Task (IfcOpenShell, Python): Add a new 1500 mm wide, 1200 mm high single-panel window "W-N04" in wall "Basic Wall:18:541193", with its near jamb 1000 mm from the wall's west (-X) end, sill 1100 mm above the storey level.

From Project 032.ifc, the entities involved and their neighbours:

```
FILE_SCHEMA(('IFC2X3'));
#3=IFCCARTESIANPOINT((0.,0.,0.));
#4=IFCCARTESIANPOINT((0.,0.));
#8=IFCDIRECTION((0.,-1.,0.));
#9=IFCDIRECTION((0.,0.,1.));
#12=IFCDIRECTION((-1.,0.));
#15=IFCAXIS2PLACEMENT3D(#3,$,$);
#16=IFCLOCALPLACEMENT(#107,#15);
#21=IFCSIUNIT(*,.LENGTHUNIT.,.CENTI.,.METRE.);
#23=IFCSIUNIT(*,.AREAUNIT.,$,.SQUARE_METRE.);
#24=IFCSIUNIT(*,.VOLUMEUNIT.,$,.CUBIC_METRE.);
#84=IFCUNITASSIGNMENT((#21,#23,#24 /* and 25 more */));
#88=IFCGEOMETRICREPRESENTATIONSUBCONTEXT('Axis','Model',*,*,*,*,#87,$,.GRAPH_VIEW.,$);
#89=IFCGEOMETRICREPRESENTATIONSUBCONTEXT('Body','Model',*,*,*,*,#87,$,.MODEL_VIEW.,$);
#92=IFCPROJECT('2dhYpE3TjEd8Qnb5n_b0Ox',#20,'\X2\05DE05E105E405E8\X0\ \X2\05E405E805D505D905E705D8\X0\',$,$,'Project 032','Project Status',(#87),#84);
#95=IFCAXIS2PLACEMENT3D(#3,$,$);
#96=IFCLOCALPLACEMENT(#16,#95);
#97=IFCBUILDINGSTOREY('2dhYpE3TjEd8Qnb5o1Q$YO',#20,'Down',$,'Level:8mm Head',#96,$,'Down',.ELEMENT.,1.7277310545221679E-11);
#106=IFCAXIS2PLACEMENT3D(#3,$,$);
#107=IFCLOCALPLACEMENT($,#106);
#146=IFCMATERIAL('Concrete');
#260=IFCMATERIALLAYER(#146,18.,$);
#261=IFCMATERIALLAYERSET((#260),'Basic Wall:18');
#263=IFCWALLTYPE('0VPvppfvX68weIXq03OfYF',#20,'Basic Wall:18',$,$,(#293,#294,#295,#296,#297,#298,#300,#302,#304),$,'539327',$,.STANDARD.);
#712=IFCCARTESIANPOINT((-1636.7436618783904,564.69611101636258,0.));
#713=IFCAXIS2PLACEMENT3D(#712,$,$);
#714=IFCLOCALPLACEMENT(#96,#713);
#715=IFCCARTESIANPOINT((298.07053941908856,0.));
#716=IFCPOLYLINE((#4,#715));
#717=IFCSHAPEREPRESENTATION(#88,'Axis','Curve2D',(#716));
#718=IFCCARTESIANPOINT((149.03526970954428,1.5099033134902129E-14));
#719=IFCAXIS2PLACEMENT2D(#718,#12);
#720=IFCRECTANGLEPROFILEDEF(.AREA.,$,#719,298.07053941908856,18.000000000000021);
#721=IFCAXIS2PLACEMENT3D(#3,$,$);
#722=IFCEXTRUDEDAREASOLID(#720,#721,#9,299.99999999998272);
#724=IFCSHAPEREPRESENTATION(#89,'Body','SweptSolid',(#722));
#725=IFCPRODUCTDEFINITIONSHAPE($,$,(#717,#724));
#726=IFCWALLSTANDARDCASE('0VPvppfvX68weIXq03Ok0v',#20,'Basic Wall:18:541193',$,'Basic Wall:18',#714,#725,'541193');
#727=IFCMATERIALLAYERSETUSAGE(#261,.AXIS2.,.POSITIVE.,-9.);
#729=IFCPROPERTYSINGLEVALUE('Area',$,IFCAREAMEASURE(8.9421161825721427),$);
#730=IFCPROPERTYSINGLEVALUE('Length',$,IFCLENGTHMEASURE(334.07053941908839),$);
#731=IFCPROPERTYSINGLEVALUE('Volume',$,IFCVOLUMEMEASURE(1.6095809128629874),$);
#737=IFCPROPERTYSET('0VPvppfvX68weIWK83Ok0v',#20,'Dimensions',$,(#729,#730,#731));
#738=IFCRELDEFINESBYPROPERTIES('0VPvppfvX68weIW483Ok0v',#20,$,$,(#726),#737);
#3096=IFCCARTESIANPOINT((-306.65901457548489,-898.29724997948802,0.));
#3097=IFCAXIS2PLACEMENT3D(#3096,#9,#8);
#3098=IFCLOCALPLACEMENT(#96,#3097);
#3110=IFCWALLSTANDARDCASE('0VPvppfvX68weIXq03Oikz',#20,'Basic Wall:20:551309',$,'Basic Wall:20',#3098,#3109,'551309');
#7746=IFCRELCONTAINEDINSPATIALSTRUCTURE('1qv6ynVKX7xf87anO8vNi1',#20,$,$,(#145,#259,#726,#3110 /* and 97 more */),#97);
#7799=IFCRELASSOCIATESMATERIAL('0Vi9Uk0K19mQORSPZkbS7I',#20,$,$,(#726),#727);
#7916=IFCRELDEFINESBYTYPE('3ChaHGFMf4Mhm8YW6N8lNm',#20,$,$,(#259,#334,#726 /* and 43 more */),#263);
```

```python
import numpy as np
import ifcopenshell
import ifcopenshell.api.feature
import ifcopenshell.api.geometry
import ifcopenshell.api.pset
import ifcopenshell.api.root
import ifcopenshell.api.spatial
import ifcopenshell.api.type
import ifcopenshell.geom
import ifcopenshell.util.element
import ifcopenshell.util.placement
import ifcopenshell.util.representation
import ifcopenshell.util.shape
import ifcopenshell.util.unit

model = ifcopenshell.open("Project 032.ifc")
unit_scale = ifcopenshell.util.unit.calculate_unit_scale(model)
area_scale = ifcopenshell.util.unit.calculate_unit_scale(model, "AREAUNIT")
volume_scale = ifcopenshell.util.unit.calculate_unit_scale(model, "VOLUMEUNIT")
settings = ifcopenshell.geom.settings()


def volume(element):
    """Net volume in cubic metres, openings subtracted."""
    shape = ifcopenshell.geom.create_shape(settings, element)
    return ifcopenshell.util.shape.get_volume(shape.geometry)


wall = model.by_id(726)
storey = ifcopenshell.util.element.get_container(wall, ifc_class="IfcBuildingStorey")
context = ifcopenshell.util.representation.get_context(model, "Model", "Body", "MODEL_VIEW")
before = volume(wall)

width, height, from_end, sill = 1.5, 1.2, 1, 1.1  # metres

# The wall runs along its own X axis, and the end named is its -X end.
wall_shape = ifcopenshell.geom.create_shape(settings, wall)
x, y, z = ifcopenshell.util.shape.get_vertices(wall_shape.geometry).T
start = x.min() + from_end
face, thickness = float(y.min()), float(y.max() - y.min())
wall_matrix = ifcopenshell.util.placement.get_local_placement(wall.ObjectPlacement)
level = ifcopenshell.util.placement.get_local_placement(storey.ObjectPlacement)[2, 3]


def in_wall(x, y):
    """Placement at x, y metres in the wall's axes, at sill height."""
    matrix = wall_matrix.copy()
    matrix[:, 3] = wall_matrix @ np.array([x / unit_scale, y / unit_scale, 0.0, 1.0])
    matrix[2, 3] = level + sill / unit_scale
    return matrix


# Opening: a box that overshoots both wall faces by 50 mm.
opening = ifcopenshell.api.root.create_entity(model, ifc_class="IfcOpeningElement")
box = ifcopenshell.api.geometry.add_wall_representation(
    model, context=context, length=width, height=height, thickness=thickness + 0.1
)
ifcopenshell.api.geometry.assign_representation(model, product=opening, representation=box)
ifcopenshell.api.geometry.edit_object_placement(model, product=opening, matrix=in_wall(start, face - 0.05), is_si=False)
ifcopenshell.api.feature.add_feature(model, feature=opening, element=wall)

window = ifcopenshell.api.root.create_entity(model, ifc_class="IfcWindow", name="W-N04")
window.OverallWidth, window.OverallHeight = width / unit_scale, height / unit_scale
body = ifcopenshell.api.geometry.add_window_representation(
    model,
    context=context,
    overall_width=window.OverallWidth,
    overall_height=window.OverallHeight,
    partition_type="SINGLE_PANEL",
)
ifcopenshell.api.geometry.assign_representation(model, product=window, representation=body)
ifcopenshell.api.spatial.assign_container(model, products=[window], relating_structure=storey)
fills = ifcopenshell.api.feature.add_filling(model, opening=opening, element=window)
fills.OwnerHistory = window.OwnerHistory  # required in IFC2X3

# IFC2X3 keeps the operation on the window style.
style = ifcopenshell.api.root.create_entity(model, ifc_class="IfcWindowStyle", name="W-N04")
style.OperationType, style.ConstructionType = "SINGLE_PANEL", "NOTDEFINED"
style.ParameterTakesPrecedence = style.Sizeable = False
ifcopenshell.api.type.assign_type(model, related_objects=[window], relating_type=style)

# Centre the window in the wall's thickness.
ifcopenshell.api.geometry.edit_object_placement(model, product=window, matrix=in_wall(start, face), is_si=False)
window_shape = ifcopenshell.geom.create_shape(settings, window)
depth = ifcopenshell.util.shape.get_vertices(window_shape.geometry)[:, 1]
offset = face + thickness / 2 - (depth.min() + depth.max()) / 2
ifcopenshell.api.geometry.edit_object_placement(model, product=window, matrix=in_wall(start, offset), is_si=False)

after = volume(wall)

# Update the wall's stored quantities.
pset = model.by_id(ifcopenshell.util.element.get_pset(wall, "Dimensions", should_inherit=False)["id"])
ifcopenshell.api.pset.edit_pset(model, pset=pset, properties={
    "Area": model.create_entity("IfcAreaMeasure", after / thickness / area_scale),
    "Volume": model.create_entity("IfcVolumeMeasure", after / volume_scale),
})

print(f"wall volume {before:.3f} -> {after:.3f} m3")

model.write("Project 032-out.ifc")
```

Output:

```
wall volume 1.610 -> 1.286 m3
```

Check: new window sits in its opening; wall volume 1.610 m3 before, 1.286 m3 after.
